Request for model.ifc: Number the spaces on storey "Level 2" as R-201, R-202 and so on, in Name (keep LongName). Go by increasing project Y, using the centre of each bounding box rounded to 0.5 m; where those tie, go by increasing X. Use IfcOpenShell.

First a look at what the model holds.

```python
import ifcopenshell
import ifcopenshell.util.element
import ifcopenshell.util.placement

model = ifcopenshell.open("model.ifc")
print(model.schema)
storey = next(s for s in model.by_type("IfcBuildingStorey") if s.Name == "Level 2")
spaces = [e for e in ifcopenshell.util.element.get_decomposition(storey) if e.is_a("IfcSpace")]
for e in sorted(spaces, key=lambda e: e.id()):
    origin = ifcopenshell.util.placement.get_local_placement(e.ObjectPlacement)[:3, 3]
    print(e.id(), e.Name, e.LongName, origin.round(2) + 0.0, sep=" | ")
```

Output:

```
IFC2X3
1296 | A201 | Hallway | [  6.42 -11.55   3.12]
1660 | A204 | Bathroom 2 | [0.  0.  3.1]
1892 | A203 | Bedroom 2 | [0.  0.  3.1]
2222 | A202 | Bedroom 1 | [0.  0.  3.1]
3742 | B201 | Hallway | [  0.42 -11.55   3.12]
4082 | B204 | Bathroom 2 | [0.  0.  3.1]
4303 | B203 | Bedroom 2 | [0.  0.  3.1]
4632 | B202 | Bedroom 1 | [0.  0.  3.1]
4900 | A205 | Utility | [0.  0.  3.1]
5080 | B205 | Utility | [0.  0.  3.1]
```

```python
import ifcopenshell
import ifcopenshell.geom
import ifcopenshell.util.element
import ifcopenshell.util.shape

model = ifcopenshell.open("model.ifc")
settings = ifcopenshell.geom.settings()
settings.set("use-world-coords", True)


def centre(element):
    shape = ifcopenshell.geom.create_shape(settings, element)
    return ifcopenshell.util.shape.get_bbox_centroid(shape.geometry)


storey = next(s for s in model.by_type("IfcBuildingStorey") if s.Name == "Level 2")
spaces = [e for e in ifcopenshell.util.element.get_decomposition(storey) if e.is_a("IfcSpace")]

# Insertion points can sit at a corner or the storey origin, so sort by the geometry (in metres).
centres = {e: centre(e) for e in spaces}
spaces.sort(key=lambda e: (round(centres[e][1] / 0.5), centres[e][0]))

for i, e in enumerate(spaces, start=1):
    number = f"R-2{i:02d}"
    e.Name = number
    print(e.id(), number)

model.write("model_rev.ifc")
```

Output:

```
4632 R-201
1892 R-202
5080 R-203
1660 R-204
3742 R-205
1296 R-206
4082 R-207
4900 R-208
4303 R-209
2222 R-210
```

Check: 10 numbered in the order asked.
